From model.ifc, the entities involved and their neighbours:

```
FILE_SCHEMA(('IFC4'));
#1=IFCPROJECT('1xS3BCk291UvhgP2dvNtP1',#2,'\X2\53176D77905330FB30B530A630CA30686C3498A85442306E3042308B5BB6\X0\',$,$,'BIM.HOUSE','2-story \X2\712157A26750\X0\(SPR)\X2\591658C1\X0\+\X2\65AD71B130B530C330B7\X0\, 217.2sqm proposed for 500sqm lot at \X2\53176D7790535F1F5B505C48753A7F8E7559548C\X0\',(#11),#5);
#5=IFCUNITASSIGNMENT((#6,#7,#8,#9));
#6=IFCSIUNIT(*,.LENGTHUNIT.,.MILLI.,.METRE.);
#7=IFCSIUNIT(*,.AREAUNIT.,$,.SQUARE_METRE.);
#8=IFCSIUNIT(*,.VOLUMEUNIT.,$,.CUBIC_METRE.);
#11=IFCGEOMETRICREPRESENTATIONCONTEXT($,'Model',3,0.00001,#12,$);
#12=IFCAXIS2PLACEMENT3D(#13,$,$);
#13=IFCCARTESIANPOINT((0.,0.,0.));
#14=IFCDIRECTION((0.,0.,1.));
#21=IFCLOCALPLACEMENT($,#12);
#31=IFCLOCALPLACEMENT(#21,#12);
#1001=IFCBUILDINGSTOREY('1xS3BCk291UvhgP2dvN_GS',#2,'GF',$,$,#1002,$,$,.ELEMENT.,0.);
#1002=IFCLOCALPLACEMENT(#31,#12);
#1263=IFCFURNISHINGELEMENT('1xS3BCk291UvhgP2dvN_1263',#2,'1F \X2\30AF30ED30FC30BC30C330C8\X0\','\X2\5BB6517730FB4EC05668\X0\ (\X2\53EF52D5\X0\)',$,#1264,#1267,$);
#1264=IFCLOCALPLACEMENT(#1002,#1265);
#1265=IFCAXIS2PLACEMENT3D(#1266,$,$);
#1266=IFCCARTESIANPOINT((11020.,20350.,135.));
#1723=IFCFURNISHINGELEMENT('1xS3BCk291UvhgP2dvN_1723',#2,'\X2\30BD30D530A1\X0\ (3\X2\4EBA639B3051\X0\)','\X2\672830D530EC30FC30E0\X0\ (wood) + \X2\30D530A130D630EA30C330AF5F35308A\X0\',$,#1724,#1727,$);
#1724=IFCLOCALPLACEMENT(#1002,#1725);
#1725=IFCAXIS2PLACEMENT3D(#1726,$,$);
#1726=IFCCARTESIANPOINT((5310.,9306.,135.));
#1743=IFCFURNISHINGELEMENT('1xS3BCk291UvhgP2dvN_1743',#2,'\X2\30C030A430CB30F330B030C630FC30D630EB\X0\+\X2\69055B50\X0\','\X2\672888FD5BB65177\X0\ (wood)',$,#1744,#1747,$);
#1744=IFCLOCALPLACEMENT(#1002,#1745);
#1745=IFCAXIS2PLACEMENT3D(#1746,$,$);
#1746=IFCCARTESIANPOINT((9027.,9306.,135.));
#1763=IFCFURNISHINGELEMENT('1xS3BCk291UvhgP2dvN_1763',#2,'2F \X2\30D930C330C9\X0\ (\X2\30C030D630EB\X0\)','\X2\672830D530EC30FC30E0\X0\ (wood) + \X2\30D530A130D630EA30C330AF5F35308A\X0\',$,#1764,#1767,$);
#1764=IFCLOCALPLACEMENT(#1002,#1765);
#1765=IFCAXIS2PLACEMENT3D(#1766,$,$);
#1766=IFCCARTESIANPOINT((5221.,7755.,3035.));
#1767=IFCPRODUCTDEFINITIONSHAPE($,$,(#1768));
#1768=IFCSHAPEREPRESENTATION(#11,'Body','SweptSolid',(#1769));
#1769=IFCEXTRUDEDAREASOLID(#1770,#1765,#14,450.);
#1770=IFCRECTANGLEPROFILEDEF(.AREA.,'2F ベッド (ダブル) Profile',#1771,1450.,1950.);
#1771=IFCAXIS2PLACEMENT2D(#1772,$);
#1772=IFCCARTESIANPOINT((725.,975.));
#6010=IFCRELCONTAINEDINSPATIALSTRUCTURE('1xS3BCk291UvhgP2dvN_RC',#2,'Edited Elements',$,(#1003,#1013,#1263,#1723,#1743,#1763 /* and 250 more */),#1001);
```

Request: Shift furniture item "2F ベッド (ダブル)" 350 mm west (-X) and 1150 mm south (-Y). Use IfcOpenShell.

```python
import ifcopenshell
import ifcopenshell.api.geometry
import ifcopenshell.util.placement
import ifcopenshell.util.unit

model = ifcopenshell.open("model.ifc")
unit_scale = ifcopenshell.util.unit.calculate_unit_scale(model)

item = model.by_id(1763)
matrix = ifcopenshell.util.placement.get_local_placement(item.ObjectPlacement)
matrix[0, 3] -= 0.35 / unit_scale
matrix[1, 3] -= 1.15 / unit_scale
ifcopenshell.api.geometry.edit_object_placement(model, product=item, matrix=matrix, is_si=False)

print(ifcopenshell.util.placement.get_local_placement(item.ObjectPlacement).round(3) + 0.0)

model.write("model_updated.ifc")
```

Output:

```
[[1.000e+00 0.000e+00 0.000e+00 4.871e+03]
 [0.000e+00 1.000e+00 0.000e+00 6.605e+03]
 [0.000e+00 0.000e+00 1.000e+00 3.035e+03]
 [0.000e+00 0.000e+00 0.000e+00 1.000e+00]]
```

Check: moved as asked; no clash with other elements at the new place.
